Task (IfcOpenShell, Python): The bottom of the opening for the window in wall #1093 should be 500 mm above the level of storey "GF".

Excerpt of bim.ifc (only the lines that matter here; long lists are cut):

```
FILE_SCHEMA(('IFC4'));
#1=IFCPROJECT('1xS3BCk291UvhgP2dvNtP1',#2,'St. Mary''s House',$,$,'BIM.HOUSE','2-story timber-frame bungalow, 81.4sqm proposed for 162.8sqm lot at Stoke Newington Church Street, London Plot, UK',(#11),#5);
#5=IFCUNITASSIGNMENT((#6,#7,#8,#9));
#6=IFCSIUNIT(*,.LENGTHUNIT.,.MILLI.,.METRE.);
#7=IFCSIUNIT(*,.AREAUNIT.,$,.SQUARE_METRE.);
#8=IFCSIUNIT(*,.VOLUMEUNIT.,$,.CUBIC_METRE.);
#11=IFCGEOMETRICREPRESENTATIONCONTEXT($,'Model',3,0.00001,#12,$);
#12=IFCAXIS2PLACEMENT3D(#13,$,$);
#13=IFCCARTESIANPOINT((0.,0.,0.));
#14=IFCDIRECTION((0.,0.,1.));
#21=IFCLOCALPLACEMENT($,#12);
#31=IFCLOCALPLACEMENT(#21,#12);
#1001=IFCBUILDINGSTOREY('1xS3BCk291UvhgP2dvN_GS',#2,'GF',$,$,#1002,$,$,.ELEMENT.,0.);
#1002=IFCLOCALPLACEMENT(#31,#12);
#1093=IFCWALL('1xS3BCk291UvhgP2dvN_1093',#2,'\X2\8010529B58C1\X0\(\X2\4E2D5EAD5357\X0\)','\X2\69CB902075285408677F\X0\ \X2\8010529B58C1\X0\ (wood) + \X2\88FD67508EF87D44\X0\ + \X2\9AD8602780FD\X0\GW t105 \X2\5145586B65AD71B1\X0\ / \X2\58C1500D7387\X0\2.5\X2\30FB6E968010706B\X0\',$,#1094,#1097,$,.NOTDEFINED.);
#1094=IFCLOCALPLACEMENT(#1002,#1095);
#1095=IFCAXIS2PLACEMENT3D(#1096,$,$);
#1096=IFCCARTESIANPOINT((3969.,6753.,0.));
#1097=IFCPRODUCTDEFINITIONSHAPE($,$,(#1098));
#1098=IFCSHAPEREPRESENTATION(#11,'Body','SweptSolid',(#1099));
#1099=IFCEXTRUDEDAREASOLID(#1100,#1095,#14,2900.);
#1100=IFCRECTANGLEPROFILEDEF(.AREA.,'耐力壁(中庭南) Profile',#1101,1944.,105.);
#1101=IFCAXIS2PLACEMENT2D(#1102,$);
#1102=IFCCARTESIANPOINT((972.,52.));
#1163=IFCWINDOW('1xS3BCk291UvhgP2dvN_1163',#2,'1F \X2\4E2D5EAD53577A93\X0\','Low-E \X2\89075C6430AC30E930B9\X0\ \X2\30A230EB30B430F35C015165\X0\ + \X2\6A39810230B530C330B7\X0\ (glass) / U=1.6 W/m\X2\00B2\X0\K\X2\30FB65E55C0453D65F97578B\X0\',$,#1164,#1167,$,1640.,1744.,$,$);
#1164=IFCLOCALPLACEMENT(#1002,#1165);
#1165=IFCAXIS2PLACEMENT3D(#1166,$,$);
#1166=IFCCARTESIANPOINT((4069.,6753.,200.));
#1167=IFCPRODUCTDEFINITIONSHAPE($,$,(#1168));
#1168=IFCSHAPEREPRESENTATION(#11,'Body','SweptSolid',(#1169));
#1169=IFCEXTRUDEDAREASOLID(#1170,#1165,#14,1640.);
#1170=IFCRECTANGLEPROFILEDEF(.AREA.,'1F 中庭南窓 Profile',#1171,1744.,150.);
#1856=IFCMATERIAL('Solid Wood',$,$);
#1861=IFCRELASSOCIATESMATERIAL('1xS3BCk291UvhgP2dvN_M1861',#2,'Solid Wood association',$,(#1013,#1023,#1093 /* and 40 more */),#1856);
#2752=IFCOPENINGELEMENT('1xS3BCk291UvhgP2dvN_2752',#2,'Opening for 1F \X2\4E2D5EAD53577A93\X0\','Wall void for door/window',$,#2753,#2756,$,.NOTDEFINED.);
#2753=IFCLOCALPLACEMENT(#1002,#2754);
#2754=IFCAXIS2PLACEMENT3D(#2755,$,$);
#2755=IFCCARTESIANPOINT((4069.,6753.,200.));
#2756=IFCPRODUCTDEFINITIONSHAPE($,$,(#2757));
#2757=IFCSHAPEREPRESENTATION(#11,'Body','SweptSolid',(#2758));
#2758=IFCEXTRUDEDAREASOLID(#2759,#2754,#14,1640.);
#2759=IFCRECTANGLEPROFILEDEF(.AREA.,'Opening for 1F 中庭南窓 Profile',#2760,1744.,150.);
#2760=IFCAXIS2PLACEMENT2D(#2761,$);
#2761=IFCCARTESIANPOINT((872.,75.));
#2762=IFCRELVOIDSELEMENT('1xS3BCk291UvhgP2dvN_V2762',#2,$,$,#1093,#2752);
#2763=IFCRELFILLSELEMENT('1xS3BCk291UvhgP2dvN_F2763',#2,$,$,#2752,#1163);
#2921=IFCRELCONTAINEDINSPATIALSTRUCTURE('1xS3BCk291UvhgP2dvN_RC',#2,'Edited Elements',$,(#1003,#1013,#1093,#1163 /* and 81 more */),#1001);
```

```python
import numpy as np
import ifcopenshell
import ifcopenshell.api.geometry
import ifcopenshell.geom
import ifcopenshell.util.element
import ifcopenshell.util.placement
import ifcopenshell.util.shape
import ifcopenshell.util.unit

model = ifcopenshell.open("bim.ifc")
unit_scale = ifcopenshell.util.unit.calculate_unit_scale(model)

window = model.by_guid("1xS3BCk291UvhgP2dvN_1163")
opening = window.FillsVoids[0].RelatingOpeningElement
storey = ifcopenshell.util.element.get_container(window, ifc_class="IfcBuildingStorey")
level = ifcopenshell.util.placement.get_local_placement(storey.ObjectPlacement)[2, 3]

# The opening's origin need not be at the sill, so measure its lowest point.
shape = ifcopenshell.geom.create_shape(ifcopenshell.geom.settings(), opening)
bottom = ifcopenshell.util.shape.get_shape_bottom_elevation(shape, shape.geometry) / unit_scale
dz = level + 0.5 / unit_scale - bottom

shift = np.array([0.0, 0.0, dz])
# The window is not placed relative to its opening, so move both.
for product in (opening, window):
    matrix = ifcopenshell.util.placement.get_local_placement(product.ObjectPlacement)
    matrix[:3, 3] += shift
    ifcopenshell.api.geometry.edit_object_placement(model, product=product, matrix=matrix, is_si=False)

print(f"moved by {dz * unit_scale:+.3f} m")

model.write("bim_rev.ifc")
```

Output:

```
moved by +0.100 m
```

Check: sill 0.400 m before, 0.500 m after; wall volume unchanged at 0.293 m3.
